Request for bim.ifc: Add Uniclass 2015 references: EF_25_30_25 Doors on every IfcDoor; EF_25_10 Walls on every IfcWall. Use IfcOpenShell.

First a look at what the model holds.

```python
import ifcopenshell

model = ifcopenshell.open("bim.ifc")
print(model.schema)
print("classifications:", [c.Name for c in model.by_type("IfcClassification")])
for ifc_class in ("IfcDoor", "IfcRoof", "IfcStair", "IfcWall", "IfcWindow"):
    print(ifc_class, len(model.by_type(ifc_class)))
```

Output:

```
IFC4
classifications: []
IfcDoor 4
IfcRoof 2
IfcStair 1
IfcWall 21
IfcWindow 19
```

```python
import ifcopenshell
import ifcopenshell.api.classification

model = ifcopenshell.open("bim.ifc")

system = ifcopenshell.api.classification.add_classification(model, classification="Uniclass 2015")

codes = {
    "IfcDoor": ("EF_25_30_25", "Doors"),
    "IfcWall": ("EF_25_10", "Walls"),
}
for ifc_class, (code, name) in codes.items():
    products = model.by_type(ifc_class)
    ifcopenshell.api.classification.add_reference(
        model, products=products, classification=system, identification=code, name=name
    )
    print(code, len(products))

model.write("bim_v2.ifc")
```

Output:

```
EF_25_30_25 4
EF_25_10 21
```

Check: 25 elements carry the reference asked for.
